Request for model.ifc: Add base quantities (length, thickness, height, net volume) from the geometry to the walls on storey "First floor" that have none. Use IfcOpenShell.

First a look at what the model holds.

```python
import ifcopenshell
import ifcopenshell.util.element
import ifcopenshell.util.unit

model = ifcopenshell.open("model.ifc")
print(model.schema)
for unit_type in ("LENGTHUNIT", "AREAUNIT", "VOLUMEUNIT"):
    print(unit_type, ifcopenshell.util.unit.calculate_unit_scale(model, unit_type))
storey = next(s for s in model.by_type("IfcBuildingStorey") if s.Name == "First floor")
walls = [e for e in ifcopenshell.util.element.get_decomposition(storey) if e.is_a("IfcWall")]
for e in sorted(walls, key=lambda e: e.id()):
    print(e.id(), e.is_a(), e.Name, list(ifcopenshell.util.element.get_psets(e, qtos_only=True)), sep=" | ")
```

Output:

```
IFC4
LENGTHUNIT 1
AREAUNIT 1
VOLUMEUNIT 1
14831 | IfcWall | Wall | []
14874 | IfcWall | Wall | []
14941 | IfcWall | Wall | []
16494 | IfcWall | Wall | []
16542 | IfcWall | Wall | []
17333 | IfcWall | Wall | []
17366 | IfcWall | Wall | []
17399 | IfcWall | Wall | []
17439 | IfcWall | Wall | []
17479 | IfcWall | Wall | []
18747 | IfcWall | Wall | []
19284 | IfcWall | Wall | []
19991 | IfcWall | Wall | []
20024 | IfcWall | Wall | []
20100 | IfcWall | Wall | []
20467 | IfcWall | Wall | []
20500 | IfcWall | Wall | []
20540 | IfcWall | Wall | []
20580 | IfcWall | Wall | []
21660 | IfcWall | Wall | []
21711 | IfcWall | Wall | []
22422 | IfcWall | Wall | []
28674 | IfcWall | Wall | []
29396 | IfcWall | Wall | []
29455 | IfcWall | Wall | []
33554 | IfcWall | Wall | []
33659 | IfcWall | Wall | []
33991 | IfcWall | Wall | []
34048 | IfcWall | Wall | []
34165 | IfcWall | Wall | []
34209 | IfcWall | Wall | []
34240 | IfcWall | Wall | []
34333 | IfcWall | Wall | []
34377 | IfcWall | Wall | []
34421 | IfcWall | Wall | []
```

```python
import ifcopenshell
import ifcopenshell.api.pset
import ifcopenshell.geom
import ifcopenshell.util.element
import ifcopenshell.util.shape
import ifcopenshell.util.unit

model = ifcopenshell.open("model.ifc")
unit_scale = ifcopenshell.util.unit.calculate_unit_scale(model)
volume_scale = ifcopenshell.util.unit.calculate_unit_scale(model, "VOLUMEUNIT")
settings = ifcopenshell.geom.settings()

storey = next(s for s in model.by_type("IfcBuildingStorey") if s.Name == "First floor")
walls = [e for e in ifcopenshell.util.element.get_decomposition(storey) if e.is_a("IfcWall")]

for e in sorted(walls, key=lambda e: e.id()):
    if ifcopenshell.util.element.get_psets(e, qtos_only=True, should_inherit=False):
        continue
    # Geometry comes back in metres, in the element's own axes.
    shape = ifcopenshell.geom.create_shape(settings, e)
    values = {
        "Length": ifcopenshell.util.shape.get_x(shape.geometry) / unit_scale,
        "Width": ifcopenshell.util.shape.get_y(shape.geometry) / unit_scale,
        "Height": ifcopenshell.util.shape.get_z(shape.geometry) / unit_scale,
        "NetVolume": ifcopenshell.util.shape.get_volume(shape.geometry) / volume_scale,
    }
    qto = ifcopenshell.api.pset.add_qto(model, product=e, name="Qto_WallBaseQuantities")
    ifcopenshell.api.pset.edit_qto(model, qto=qto, properties=values)
    print(e.id(), {k: round(v, 3) for k, v in values.items()})

model.write("model-out.ifc")
```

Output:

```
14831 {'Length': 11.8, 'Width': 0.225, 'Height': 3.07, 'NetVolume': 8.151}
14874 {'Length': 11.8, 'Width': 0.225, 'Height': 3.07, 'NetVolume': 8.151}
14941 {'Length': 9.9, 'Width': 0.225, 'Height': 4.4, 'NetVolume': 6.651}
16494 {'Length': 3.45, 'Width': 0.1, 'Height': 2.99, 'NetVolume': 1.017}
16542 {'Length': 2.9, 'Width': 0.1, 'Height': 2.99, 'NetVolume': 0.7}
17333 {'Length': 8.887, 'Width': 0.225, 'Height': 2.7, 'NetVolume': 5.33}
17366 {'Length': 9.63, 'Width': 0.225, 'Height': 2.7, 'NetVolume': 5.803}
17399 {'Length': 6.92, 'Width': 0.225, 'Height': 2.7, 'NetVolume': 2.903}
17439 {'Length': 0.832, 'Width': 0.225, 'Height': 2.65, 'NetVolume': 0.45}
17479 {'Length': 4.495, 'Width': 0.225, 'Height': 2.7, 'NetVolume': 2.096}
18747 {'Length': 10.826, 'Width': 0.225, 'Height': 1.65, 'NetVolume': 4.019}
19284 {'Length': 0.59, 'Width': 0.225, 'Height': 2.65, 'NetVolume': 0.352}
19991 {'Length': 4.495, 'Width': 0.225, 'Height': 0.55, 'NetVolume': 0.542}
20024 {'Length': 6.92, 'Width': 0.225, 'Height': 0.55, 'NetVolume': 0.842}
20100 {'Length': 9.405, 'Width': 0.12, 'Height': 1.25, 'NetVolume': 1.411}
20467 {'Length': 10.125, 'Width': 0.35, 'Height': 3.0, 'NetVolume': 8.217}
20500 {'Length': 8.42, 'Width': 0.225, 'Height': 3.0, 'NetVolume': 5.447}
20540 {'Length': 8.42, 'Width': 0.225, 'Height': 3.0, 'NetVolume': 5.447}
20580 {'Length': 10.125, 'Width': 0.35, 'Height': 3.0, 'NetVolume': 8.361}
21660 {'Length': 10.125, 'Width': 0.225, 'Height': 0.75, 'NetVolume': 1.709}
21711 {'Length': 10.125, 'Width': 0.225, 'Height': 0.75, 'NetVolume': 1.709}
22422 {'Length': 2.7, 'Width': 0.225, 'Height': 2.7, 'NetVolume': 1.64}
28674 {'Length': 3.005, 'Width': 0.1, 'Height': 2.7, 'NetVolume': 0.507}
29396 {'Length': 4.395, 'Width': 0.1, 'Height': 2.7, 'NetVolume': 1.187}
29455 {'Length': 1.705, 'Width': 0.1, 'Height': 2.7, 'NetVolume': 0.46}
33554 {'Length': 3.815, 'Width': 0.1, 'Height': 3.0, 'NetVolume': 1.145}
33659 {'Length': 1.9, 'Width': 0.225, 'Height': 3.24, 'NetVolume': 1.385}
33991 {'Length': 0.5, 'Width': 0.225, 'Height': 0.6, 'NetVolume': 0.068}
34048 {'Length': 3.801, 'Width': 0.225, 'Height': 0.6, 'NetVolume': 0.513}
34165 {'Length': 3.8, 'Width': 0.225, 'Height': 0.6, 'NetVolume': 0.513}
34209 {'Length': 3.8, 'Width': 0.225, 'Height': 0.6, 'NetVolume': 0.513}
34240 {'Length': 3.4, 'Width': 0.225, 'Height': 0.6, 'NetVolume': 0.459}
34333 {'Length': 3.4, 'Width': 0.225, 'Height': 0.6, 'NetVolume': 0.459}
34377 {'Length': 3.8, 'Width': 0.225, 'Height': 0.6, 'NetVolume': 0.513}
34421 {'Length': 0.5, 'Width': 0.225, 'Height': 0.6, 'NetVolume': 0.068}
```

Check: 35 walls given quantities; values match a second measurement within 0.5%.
